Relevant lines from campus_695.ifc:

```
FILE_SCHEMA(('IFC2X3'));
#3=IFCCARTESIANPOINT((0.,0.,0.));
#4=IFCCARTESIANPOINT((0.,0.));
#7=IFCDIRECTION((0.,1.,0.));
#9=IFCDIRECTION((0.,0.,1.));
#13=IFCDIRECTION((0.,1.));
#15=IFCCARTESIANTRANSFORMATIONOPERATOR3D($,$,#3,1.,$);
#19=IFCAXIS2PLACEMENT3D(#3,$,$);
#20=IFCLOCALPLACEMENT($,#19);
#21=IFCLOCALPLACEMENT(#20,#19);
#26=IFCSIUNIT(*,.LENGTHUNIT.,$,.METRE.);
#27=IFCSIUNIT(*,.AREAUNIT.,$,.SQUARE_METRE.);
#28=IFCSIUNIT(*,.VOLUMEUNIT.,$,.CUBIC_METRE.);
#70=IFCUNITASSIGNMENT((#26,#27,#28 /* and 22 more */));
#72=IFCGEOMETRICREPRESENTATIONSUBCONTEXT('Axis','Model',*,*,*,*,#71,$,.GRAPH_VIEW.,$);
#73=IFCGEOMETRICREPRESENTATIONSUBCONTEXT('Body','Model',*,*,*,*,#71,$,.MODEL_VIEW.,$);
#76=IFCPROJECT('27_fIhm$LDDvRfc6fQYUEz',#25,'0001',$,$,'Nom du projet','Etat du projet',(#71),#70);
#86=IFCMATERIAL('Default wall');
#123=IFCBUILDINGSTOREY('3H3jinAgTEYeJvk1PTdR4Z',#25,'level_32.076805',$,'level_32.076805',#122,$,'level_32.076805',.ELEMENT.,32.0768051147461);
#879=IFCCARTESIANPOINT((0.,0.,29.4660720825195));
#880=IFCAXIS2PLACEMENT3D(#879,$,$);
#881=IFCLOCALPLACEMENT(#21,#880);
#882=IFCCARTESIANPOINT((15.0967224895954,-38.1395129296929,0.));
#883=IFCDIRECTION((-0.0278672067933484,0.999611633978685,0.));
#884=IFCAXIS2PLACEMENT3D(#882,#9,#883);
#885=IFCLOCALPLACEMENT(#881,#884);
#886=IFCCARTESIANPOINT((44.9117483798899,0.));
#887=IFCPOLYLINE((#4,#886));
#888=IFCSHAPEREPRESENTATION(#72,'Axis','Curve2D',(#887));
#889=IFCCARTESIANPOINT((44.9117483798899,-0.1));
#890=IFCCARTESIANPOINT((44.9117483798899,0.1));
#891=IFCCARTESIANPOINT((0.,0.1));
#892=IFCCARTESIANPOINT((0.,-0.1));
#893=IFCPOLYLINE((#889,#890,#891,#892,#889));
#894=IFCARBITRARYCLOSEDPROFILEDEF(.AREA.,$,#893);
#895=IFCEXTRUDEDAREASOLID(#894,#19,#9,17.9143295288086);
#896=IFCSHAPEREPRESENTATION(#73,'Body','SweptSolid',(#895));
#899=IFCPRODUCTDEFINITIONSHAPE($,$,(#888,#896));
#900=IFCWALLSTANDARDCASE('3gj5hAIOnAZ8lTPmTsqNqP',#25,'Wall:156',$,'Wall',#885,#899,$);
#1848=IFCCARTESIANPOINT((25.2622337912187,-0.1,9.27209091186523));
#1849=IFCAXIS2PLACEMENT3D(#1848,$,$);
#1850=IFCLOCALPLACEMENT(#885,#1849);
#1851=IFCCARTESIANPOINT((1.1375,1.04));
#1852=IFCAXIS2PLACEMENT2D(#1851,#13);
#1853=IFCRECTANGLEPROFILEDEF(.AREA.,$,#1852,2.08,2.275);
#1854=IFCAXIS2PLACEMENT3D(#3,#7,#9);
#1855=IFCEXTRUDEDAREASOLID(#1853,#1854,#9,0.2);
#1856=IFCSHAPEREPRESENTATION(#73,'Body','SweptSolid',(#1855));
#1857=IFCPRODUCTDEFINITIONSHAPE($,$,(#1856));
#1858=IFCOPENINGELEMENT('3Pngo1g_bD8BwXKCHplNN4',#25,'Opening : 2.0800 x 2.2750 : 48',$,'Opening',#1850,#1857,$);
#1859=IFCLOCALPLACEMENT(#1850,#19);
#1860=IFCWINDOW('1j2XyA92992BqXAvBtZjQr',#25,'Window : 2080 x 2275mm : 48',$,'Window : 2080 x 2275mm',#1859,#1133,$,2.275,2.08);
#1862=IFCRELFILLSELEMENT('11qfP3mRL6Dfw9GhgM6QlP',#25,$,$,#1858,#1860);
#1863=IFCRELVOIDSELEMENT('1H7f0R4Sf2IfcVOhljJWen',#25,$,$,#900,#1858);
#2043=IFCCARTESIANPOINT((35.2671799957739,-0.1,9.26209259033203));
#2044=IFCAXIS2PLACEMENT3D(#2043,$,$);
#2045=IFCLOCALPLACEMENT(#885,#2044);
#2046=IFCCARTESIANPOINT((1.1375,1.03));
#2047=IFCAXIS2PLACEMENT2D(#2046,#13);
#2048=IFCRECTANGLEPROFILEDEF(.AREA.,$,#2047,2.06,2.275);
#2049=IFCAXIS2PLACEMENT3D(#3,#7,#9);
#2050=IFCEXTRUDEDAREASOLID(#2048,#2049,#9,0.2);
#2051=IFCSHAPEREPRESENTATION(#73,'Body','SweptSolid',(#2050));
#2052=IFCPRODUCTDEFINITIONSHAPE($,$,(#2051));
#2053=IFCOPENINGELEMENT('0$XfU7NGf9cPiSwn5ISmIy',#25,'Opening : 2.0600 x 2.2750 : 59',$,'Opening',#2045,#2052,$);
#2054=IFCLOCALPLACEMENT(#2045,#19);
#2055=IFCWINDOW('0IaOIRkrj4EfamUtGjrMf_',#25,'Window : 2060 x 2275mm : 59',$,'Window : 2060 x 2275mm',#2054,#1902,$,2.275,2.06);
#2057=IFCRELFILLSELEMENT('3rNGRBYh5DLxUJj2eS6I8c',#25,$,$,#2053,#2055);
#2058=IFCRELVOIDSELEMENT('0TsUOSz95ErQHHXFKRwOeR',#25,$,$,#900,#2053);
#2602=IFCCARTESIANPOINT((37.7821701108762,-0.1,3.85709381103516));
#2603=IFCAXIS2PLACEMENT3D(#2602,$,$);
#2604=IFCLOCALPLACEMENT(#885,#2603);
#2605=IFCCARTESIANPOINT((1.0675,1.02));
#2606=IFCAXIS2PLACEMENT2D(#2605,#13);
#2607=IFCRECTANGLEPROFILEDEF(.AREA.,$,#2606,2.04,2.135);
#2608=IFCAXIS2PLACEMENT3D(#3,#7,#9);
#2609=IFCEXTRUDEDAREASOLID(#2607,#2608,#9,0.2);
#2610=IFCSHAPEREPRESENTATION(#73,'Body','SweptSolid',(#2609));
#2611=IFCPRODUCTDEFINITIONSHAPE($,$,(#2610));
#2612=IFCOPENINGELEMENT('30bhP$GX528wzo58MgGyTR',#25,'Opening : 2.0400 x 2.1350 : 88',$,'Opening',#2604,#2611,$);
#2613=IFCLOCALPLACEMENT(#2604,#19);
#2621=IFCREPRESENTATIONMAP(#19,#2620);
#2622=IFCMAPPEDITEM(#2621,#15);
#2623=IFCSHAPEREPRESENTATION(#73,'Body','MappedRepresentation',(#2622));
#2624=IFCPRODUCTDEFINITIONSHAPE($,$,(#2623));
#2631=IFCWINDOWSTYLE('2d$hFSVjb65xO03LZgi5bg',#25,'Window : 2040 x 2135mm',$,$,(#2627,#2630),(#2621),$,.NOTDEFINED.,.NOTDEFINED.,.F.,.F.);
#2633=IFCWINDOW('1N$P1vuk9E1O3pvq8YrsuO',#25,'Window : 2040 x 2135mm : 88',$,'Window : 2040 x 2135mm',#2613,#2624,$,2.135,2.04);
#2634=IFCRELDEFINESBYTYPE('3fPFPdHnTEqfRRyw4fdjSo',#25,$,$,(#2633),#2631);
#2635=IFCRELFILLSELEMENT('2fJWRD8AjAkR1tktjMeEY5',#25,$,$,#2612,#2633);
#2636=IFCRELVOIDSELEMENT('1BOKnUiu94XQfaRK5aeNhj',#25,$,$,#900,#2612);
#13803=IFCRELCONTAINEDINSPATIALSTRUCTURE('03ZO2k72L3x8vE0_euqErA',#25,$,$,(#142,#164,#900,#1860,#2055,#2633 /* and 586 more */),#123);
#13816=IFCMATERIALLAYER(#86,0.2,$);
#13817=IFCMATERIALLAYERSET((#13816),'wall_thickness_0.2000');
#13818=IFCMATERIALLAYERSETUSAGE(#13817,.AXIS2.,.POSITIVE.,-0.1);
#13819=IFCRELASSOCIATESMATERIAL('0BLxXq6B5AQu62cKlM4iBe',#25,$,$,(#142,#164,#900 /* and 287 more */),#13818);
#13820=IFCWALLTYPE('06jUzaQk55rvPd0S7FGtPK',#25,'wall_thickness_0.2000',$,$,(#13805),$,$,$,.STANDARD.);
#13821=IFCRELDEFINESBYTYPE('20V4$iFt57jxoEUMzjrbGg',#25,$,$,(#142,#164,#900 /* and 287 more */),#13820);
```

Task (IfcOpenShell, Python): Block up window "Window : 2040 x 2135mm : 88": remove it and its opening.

```python
import ifcopenshell
import ifcopenshell.api.feature
import ifcopenshell.api.root
import ifcopenshell.geom
import ifcopenshell.util.shape

model = ifcopenshell.open("campus_695.ifc")
settings = ifcopenshell.geom.settings()


def volume(element):
    """Net volume in cubic metres, openings subtracted."""
    shape = ifcopenshell.geom.create_shape(settings, element)
    return ifcopenshell.util.shape.get_volume(shape.geometry)


window = model.by_guid("1N$P1vuk9E1O3pvq8YrsuO")
opening = window.FillsVoids[0].RelatingOpeningElement
wall = opening.VoidsElements[0].RelatingBuildingElement
before = volume(wall)

ifcopenshell.api.root.remove_product(model, product=window)
ifcopenshell.api.feature.remove_feature(model, feature=opening)

after = volume(wall)

print(f"wall volume {before:.3f} -> {after:.3f} m3")

model.write("campus_695_edited.ifc")
```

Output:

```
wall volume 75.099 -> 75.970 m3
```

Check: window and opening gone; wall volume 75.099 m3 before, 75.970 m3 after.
